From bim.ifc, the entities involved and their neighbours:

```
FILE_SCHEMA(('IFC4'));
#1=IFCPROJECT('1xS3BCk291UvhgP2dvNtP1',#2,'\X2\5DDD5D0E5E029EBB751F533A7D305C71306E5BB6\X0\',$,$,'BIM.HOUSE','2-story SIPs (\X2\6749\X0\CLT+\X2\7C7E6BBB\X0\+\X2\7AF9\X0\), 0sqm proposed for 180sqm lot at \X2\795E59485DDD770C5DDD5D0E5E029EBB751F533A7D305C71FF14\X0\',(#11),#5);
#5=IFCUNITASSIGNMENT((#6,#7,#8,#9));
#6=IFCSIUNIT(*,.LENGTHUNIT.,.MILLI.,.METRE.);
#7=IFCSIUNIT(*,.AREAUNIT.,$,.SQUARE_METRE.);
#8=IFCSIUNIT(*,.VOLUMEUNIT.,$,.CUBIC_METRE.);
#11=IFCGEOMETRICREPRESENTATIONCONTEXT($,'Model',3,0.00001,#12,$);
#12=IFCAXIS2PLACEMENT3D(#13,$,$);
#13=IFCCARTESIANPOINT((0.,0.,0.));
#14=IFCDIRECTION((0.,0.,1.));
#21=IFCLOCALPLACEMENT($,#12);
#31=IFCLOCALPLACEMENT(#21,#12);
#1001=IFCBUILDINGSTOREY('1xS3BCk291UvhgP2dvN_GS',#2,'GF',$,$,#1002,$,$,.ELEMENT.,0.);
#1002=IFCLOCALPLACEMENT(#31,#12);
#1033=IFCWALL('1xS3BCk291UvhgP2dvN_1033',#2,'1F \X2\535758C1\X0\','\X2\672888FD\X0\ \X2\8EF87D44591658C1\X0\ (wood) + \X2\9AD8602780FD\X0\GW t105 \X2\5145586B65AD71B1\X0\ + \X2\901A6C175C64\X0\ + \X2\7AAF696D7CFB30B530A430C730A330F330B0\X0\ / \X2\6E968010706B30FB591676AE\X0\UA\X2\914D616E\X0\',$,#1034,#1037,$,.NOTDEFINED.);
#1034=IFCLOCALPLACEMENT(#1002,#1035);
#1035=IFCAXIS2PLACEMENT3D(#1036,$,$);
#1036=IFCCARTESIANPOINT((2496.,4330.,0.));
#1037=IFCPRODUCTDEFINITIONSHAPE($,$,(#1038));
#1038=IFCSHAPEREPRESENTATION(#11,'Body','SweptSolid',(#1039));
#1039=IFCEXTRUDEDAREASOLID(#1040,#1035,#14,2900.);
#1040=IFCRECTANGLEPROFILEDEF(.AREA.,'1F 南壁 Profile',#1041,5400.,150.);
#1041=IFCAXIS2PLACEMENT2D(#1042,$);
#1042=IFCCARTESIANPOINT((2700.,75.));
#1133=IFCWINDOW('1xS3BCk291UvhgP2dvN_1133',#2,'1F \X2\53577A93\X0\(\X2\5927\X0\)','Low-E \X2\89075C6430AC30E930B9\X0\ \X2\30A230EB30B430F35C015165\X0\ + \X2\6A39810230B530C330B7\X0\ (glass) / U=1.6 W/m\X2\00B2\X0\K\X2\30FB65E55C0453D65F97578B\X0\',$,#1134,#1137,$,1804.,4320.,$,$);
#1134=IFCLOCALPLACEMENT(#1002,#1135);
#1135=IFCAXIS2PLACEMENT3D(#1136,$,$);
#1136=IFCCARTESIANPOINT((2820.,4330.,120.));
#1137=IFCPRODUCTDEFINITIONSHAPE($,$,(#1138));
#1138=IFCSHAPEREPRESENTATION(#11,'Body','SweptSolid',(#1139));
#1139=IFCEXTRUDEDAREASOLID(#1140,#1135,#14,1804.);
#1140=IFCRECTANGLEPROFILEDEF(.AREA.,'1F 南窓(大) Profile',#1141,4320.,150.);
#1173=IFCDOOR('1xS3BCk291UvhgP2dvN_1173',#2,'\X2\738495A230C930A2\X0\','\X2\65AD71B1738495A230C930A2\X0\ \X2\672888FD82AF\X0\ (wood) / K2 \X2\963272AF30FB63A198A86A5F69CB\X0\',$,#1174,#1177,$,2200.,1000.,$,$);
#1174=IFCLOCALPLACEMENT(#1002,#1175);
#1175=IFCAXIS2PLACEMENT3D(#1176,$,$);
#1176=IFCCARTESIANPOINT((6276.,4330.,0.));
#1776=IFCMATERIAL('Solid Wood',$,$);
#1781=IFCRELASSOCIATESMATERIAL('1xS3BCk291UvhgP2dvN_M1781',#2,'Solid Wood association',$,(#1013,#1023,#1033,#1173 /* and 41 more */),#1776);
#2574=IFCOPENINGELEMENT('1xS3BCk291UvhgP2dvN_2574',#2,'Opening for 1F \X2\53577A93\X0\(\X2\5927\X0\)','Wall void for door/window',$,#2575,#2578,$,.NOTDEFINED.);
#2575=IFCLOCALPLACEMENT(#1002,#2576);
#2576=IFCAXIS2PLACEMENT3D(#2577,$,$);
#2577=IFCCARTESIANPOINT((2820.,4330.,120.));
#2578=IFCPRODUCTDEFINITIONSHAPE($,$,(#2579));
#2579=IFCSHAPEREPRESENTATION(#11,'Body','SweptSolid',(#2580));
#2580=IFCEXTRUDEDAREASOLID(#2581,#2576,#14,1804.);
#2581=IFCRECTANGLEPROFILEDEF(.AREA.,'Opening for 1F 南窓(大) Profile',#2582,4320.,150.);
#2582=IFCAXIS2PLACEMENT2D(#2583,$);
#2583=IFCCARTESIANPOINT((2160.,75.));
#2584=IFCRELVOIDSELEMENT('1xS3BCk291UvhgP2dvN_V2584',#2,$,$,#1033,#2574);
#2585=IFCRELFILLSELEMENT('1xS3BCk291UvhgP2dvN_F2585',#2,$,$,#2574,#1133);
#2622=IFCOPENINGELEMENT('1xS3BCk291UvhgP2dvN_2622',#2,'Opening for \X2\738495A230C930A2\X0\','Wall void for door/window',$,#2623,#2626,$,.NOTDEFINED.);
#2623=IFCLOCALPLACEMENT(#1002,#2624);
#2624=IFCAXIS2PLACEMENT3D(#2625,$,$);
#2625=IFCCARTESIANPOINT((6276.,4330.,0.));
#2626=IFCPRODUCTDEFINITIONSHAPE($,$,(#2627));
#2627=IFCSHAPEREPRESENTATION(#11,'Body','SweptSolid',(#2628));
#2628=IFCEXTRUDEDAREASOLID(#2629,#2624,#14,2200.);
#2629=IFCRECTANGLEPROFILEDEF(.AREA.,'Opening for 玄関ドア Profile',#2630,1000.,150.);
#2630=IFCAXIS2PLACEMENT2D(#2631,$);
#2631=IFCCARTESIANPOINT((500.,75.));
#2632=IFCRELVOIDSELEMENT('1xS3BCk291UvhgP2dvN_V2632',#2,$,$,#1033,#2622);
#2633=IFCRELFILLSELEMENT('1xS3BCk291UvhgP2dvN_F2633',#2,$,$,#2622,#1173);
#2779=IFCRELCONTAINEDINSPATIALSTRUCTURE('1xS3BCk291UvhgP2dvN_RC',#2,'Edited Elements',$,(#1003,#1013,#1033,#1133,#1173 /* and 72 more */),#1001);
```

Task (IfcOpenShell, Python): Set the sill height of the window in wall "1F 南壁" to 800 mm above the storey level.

```python
import numpy as np
import ifcopenshell
import ifcopenshell.api.geometry
import ifcopenshell.geom
import ifcopenshell.util.element
import ifcopenshell.util.placement
import ifcopenshell.util.shape
import ifcopenshell.util.unit

model = ifcopenshell.open("bim.ifc")
unit_scale = ifcopenshell.util.unit.calculate_unit_scale(model)

window = model.by_guid("1xS3BCk291UvhgP2dvN_1133")
opening = window.FillsVoids[0].RelatingOpeningElement
storey = ifcopenshell.util.element.get_container(window, ifc_class="IfcBuildingStorey")
level = ifcopenshell.util.placement.get_local_placement(storey.ObjectPlacement)[2, 3]

# The opening's origin need not be at the sill, so measure its lowest point.
shape = ifcopenshell.geom.create_shape(ifcopenshell.geom.settings(), opening)
bottom = ifcopenshell.util.shape.get_shape_bottom_elevation(shape, shape.geometry) / unit_scale
dz = level + 800.0 - bottom

shift = np.array([0.0, 0.0, dz])
# The window is not placed relative to its opening, so move both.
for product in (opening, window):
    matrix = ifcopenshell.util.placement.get_local_placement(product.ObjectPlacement)
    matrix[:3, 3] += shift
    ifcopenshell.api.geometry.edit_object_placement(model, product=product, matrix=matrix, is_si=False)

print(f"moved by {dz * unit_scale:+.3f} m")

model.write("bim_edited.ifc")
```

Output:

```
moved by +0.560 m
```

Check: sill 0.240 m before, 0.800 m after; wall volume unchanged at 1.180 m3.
